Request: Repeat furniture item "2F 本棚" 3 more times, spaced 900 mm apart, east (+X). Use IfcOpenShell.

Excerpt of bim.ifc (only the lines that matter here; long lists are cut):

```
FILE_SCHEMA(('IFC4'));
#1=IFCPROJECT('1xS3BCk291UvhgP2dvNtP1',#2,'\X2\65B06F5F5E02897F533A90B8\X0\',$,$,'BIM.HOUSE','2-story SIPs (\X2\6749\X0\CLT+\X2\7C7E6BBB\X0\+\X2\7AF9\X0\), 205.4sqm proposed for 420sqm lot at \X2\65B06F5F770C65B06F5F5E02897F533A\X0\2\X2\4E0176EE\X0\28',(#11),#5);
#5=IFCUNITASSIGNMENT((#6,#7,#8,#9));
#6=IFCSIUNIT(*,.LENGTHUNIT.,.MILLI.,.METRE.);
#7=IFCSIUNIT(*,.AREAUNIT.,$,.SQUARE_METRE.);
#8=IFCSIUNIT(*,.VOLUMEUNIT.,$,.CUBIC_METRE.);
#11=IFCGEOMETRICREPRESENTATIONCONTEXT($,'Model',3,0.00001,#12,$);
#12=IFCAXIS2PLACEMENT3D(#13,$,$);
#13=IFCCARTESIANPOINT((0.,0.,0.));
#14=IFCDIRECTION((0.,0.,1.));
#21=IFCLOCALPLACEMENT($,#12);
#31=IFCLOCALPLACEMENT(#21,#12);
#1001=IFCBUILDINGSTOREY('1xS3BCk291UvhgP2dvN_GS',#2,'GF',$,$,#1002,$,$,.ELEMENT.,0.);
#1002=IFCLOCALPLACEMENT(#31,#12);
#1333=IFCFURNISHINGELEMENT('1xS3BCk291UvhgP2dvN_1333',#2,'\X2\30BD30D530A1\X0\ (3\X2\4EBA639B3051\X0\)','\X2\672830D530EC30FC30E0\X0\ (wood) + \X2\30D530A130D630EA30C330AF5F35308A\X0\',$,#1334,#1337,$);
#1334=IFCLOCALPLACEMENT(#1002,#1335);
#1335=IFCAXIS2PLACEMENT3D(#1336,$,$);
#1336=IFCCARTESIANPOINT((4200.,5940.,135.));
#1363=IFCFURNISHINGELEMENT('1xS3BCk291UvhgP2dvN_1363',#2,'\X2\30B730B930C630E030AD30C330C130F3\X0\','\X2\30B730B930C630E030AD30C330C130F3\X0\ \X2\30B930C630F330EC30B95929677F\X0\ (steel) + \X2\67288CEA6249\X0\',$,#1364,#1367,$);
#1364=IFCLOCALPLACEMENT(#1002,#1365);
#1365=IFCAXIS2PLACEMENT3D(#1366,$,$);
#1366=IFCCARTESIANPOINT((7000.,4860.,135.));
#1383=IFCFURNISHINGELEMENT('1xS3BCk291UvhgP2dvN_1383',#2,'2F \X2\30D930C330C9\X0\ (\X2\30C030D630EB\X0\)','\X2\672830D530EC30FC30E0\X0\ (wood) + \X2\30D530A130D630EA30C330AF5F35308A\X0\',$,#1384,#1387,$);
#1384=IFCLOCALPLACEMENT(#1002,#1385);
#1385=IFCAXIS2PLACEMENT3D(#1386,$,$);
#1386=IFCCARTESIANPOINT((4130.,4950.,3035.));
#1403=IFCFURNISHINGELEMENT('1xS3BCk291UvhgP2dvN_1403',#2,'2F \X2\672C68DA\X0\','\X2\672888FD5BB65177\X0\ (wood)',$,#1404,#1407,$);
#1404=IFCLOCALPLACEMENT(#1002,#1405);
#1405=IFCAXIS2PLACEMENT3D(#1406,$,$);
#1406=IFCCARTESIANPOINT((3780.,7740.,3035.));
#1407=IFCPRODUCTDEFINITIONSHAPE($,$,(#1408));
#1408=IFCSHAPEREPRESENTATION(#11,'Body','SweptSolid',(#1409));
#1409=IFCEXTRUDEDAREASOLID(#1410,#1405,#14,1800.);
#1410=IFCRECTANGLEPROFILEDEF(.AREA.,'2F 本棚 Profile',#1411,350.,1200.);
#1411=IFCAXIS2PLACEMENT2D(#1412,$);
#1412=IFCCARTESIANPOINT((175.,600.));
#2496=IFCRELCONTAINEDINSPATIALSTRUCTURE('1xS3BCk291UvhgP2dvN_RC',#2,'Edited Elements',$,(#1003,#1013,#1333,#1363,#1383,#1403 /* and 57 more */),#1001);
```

```python
import numpy as np
import ifcopenshell
import ifcopenshell.api.geometry
import ifcopenshell.api.root
import ifcopenshell.util.element
import ifcopenshell.util.placement

model = ifcopenshell.open("bim.ifc")


def reuse_history(source, copy):
    """copy_class also copies each property set's owner history, people and application; keep the originals."""
    for rel in copy.IsDefinedBy:
        if rel.is_a("IfcRelDefinesByProperties") and (history := rel.RelatingPropertyDefinition.OwnerHistory):
            rel.RelatingPropertyDefinition.OwnerHistory = source.OwnerHistory
            ifcopenshell.util.element.remove_deep2(model, history)


source = model.by_guid("1xS3BCk291UvhgP2dvN_1403")
base = ifcopenshell.util.placement.get_local_placement(source.ObjectPlacement)
step = np.array([1.0, 0.0, 0.0]) * 900.0

for i in range(1, 4):
    copy = ifcopenshell.api.root.copy_class(model, product=source)
    copy.Representation = ifcopenshell.util.element.copy_deep(
        model, source.Representation, exclude=["IfcGeometricRepresentationContext", "IfcRepresentationMap"]
    )
    reuse_history(source, copy)
    matrix = base.copy()
    matrix[:3, 3] += i * step
    print("added at", matrix[:3, 3].round(3) + 0.0)
    ifcopenshell.api.geometry.edit_object_placement(model, product=copy, matrix=matrix, is_si=False)

model.write("bim-out.ifc")
```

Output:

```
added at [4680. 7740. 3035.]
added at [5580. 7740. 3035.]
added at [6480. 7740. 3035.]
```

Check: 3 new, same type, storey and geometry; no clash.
